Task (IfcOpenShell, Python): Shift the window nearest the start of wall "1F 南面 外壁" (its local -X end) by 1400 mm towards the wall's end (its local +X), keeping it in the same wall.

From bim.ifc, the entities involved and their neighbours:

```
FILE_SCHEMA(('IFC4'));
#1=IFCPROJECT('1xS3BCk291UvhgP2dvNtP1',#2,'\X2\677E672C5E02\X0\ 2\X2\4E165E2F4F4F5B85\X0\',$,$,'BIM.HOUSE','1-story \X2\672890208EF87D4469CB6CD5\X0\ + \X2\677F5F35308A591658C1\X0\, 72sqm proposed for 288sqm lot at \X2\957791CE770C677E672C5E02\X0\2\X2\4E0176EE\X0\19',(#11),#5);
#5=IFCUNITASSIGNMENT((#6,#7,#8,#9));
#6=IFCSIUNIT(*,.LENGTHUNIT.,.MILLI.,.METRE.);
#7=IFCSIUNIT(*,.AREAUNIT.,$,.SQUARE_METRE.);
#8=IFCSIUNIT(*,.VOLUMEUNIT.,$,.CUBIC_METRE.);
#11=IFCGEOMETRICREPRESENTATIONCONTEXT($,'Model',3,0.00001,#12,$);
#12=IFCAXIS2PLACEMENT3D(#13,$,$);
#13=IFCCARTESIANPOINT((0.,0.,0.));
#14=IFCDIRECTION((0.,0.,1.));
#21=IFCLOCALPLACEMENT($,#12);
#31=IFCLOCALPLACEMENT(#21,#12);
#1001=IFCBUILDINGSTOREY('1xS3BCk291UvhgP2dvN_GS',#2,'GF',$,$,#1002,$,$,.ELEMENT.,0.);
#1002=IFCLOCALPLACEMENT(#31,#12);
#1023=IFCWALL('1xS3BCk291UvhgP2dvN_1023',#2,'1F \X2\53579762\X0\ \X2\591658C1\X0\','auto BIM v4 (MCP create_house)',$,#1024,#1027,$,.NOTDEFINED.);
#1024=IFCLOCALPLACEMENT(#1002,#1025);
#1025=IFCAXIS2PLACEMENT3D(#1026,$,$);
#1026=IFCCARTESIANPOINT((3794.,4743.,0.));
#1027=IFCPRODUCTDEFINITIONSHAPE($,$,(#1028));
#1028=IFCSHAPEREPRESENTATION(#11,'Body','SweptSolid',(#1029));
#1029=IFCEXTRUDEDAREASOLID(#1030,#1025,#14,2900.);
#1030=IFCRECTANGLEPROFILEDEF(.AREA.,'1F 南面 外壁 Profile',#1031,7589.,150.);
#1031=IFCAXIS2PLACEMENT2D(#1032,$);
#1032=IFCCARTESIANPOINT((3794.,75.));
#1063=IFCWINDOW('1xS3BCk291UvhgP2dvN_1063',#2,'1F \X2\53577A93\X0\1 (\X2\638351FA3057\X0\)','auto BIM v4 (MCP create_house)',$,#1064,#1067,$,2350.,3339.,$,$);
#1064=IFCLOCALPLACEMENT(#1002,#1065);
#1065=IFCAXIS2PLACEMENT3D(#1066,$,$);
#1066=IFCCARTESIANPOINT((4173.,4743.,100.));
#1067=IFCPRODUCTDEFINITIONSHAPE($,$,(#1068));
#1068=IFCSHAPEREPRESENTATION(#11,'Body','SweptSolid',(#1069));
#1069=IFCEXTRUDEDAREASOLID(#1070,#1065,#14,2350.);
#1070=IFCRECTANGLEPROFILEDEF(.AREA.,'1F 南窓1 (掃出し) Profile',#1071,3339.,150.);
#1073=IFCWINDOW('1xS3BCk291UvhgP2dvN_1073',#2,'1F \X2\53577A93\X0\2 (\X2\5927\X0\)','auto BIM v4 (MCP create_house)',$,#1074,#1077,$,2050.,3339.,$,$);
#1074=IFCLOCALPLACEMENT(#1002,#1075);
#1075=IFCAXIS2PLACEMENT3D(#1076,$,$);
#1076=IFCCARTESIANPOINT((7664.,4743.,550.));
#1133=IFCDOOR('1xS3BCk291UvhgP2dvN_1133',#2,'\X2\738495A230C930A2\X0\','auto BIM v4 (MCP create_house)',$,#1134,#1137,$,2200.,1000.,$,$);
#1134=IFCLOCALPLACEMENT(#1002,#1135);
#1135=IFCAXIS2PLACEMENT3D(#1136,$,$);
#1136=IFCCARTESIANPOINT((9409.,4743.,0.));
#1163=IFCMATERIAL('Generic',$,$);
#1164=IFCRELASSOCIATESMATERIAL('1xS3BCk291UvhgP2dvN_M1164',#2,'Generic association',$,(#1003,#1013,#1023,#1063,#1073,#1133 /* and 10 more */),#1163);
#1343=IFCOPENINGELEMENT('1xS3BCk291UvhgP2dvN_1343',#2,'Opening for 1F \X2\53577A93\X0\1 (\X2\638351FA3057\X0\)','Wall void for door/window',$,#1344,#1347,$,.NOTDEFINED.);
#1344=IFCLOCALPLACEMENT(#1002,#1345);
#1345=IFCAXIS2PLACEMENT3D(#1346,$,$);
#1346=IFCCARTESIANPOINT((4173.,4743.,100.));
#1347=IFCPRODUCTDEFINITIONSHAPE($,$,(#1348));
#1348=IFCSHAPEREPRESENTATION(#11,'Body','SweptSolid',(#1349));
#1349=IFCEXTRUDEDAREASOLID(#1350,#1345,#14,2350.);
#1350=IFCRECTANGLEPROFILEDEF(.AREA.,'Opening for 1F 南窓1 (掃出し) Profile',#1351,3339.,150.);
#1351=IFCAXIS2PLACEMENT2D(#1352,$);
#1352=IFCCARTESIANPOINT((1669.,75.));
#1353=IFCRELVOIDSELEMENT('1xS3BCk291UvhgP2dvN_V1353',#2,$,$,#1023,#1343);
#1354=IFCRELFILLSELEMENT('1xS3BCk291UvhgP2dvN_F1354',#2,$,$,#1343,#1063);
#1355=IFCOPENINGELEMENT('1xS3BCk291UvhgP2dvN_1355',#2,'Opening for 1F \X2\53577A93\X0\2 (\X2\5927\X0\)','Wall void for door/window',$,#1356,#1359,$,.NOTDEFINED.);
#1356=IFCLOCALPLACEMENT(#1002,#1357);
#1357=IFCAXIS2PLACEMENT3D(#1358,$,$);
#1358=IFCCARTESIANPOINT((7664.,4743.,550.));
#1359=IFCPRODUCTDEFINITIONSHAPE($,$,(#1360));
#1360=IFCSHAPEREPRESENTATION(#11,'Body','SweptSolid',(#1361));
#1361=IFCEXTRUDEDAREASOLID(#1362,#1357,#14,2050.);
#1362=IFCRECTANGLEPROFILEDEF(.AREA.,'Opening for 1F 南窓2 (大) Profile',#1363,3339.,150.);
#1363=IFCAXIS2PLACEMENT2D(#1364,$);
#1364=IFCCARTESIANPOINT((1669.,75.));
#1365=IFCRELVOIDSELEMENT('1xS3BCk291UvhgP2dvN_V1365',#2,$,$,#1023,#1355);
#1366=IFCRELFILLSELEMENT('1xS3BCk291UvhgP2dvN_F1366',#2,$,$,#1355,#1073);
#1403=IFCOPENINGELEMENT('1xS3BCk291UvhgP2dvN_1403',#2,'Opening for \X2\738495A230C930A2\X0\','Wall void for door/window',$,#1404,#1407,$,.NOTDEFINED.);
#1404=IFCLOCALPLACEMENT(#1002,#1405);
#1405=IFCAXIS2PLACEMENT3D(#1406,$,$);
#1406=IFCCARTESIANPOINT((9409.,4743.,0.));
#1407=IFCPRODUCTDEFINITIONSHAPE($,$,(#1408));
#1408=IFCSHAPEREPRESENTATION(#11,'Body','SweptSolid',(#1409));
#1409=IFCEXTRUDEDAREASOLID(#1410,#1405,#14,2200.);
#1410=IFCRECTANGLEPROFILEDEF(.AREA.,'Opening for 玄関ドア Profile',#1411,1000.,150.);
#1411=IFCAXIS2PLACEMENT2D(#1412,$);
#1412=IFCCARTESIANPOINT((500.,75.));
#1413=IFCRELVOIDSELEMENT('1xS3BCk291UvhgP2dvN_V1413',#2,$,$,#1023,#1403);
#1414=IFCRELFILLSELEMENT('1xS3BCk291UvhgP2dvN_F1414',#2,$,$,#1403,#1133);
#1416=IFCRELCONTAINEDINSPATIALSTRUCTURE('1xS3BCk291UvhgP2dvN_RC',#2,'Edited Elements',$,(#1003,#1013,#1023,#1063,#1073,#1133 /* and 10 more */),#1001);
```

```python
import ifcopenshell
import ifcopenshell.api.geometry
import ifcopenshell.util.placement
import ifcopenshell.util.unit

model = ifcopenshell.open("bim.ifc")
unit_scale = ifcopenshell.util.unit.calculate_unit_scale(model)

window = model.by_guid("1xS3BCk291UvhgP2dvN_1063")
opening = window.FillsVoids[0].RelatingOpeningElement
wall = opening.VoidsElements[0].RelatingBuildingElement

wall_matrix = ifcopenshell.util.placement.get_local_placement(wall.ObjectPlacement)
shift = wall_matrix[:3, 0] * 1.4 / unit_scale
before = ifcopenshell.util.placement.get_local_placement(window.ObjectPlacement)[:3, 3].copy()

# The window is not placed relative to its opening, so move both.
for product in (opening, window):
    matrix = ifcopenshell.util.placement.get_local_placement(product.ObjectPlacement)
    matrix[:3, 3] += shift
    ifcopenshell.api.geometry.edit_object_placement(model, product=product, matrix=matrix, is_si=False)

after = ifcopenshell.util.placement.get_local_placement(window.ObjectPlacement)[:3, 3]
print("window moved by", (after - before).round(3) + 0.0)

model.write("bim-out.ifc")
```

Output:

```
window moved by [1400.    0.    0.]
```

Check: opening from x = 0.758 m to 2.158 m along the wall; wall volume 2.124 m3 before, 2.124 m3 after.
